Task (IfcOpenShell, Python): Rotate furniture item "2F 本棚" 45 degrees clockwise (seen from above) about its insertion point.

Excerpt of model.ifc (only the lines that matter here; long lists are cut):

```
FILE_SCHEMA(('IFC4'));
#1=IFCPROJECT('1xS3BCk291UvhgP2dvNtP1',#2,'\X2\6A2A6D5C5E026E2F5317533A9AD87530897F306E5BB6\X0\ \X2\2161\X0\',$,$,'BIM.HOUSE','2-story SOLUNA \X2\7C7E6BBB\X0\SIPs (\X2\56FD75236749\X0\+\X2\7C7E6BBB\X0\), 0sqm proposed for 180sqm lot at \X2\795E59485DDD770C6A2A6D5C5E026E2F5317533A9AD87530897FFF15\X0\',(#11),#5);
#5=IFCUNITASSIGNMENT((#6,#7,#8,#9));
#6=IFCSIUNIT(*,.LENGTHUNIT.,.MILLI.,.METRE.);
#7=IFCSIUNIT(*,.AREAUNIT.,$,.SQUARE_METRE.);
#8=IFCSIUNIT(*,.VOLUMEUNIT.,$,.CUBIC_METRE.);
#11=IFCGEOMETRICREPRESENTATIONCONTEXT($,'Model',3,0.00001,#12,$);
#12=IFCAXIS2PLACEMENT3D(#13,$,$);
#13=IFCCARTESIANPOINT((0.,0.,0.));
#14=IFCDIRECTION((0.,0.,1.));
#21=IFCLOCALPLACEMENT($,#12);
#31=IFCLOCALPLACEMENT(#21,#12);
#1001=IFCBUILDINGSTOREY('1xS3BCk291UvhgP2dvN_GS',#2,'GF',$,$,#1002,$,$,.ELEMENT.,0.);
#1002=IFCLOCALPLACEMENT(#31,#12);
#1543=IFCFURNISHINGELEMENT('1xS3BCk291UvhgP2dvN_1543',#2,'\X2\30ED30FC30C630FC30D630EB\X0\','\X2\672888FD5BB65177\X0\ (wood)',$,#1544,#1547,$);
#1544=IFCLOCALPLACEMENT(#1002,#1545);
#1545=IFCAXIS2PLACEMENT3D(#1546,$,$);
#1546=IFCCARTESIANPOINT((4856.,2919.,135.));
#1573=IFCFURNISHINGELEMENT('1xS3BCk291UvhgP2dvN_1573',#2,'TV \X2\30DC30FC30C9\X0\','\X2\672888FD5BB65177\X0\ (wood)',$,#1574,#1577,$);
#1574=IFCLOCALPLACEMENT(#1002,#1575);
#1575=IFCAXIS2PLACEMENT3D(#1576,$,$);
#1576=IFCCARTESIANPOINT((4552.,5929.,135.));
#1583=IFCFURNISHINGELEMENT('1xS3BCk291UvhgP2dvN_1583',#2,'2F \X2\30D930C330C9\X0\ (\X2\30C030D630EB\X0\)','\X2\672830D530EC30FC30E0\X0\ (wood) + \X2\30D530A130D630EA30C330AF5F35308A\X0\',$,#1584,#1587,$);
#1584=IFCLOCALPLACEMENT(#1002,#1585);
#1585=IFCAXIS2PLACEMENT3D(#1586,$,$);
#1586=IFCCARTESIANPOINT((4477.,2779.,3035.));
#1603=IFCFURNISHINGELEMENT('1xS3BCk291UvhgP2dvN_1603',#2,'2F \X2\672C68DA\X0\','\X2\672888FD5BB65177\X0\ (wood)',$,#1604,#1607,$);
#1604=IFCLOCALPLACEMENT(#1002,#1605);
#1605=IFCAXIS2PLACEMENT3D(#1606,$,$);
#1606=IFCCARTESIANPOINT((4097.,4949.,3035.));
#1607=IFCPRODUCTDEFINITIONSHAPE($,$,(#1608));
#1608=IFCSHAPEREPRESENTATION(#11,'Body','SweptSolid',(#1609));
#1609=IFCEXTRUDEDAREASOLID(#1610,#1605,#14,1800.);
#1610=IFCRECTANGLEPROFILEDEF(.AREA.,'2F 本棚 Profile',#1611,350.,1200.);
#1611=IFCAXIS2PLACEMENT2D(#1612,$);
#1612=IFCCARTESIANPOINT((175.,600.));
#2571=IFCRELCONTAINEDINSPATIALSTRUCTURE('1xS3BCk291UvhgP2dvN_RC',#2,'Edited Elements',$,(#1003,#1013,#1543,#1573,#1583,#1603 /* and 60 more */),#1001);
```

```python
import ifcopenshell
import ifcopenshell.api.geometry
import ifcopenshell.util.placement

model = ifcopenshell.open("model.ifc")

item = model.by_guid("1xS3BCk291UvhgP2dvN_1603")
matrix = ifcopenshell.util.placement.get_local_placement(item.ObjectPlacement)
matrix = matrix @ ifcopenshell.util.placement.rotation(-45, "Z")
ifcopenshell.api.geometry.edit_object_placement(model, product=item, matrix=matrix, is_si=False)

print(ifcopenshell.util.placement.get_local_placement(item.ObjectPlacement).round(3) + 0.0)

model.write("model_v2.ifc")
```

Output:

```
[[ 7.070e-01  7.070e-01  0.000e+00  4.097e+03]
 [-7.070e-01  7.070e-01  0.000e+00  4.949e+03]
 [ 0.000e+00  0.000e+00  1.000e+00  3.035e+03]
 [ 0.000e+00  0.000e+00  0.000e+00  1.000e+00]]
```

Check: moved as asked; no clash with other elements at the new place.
